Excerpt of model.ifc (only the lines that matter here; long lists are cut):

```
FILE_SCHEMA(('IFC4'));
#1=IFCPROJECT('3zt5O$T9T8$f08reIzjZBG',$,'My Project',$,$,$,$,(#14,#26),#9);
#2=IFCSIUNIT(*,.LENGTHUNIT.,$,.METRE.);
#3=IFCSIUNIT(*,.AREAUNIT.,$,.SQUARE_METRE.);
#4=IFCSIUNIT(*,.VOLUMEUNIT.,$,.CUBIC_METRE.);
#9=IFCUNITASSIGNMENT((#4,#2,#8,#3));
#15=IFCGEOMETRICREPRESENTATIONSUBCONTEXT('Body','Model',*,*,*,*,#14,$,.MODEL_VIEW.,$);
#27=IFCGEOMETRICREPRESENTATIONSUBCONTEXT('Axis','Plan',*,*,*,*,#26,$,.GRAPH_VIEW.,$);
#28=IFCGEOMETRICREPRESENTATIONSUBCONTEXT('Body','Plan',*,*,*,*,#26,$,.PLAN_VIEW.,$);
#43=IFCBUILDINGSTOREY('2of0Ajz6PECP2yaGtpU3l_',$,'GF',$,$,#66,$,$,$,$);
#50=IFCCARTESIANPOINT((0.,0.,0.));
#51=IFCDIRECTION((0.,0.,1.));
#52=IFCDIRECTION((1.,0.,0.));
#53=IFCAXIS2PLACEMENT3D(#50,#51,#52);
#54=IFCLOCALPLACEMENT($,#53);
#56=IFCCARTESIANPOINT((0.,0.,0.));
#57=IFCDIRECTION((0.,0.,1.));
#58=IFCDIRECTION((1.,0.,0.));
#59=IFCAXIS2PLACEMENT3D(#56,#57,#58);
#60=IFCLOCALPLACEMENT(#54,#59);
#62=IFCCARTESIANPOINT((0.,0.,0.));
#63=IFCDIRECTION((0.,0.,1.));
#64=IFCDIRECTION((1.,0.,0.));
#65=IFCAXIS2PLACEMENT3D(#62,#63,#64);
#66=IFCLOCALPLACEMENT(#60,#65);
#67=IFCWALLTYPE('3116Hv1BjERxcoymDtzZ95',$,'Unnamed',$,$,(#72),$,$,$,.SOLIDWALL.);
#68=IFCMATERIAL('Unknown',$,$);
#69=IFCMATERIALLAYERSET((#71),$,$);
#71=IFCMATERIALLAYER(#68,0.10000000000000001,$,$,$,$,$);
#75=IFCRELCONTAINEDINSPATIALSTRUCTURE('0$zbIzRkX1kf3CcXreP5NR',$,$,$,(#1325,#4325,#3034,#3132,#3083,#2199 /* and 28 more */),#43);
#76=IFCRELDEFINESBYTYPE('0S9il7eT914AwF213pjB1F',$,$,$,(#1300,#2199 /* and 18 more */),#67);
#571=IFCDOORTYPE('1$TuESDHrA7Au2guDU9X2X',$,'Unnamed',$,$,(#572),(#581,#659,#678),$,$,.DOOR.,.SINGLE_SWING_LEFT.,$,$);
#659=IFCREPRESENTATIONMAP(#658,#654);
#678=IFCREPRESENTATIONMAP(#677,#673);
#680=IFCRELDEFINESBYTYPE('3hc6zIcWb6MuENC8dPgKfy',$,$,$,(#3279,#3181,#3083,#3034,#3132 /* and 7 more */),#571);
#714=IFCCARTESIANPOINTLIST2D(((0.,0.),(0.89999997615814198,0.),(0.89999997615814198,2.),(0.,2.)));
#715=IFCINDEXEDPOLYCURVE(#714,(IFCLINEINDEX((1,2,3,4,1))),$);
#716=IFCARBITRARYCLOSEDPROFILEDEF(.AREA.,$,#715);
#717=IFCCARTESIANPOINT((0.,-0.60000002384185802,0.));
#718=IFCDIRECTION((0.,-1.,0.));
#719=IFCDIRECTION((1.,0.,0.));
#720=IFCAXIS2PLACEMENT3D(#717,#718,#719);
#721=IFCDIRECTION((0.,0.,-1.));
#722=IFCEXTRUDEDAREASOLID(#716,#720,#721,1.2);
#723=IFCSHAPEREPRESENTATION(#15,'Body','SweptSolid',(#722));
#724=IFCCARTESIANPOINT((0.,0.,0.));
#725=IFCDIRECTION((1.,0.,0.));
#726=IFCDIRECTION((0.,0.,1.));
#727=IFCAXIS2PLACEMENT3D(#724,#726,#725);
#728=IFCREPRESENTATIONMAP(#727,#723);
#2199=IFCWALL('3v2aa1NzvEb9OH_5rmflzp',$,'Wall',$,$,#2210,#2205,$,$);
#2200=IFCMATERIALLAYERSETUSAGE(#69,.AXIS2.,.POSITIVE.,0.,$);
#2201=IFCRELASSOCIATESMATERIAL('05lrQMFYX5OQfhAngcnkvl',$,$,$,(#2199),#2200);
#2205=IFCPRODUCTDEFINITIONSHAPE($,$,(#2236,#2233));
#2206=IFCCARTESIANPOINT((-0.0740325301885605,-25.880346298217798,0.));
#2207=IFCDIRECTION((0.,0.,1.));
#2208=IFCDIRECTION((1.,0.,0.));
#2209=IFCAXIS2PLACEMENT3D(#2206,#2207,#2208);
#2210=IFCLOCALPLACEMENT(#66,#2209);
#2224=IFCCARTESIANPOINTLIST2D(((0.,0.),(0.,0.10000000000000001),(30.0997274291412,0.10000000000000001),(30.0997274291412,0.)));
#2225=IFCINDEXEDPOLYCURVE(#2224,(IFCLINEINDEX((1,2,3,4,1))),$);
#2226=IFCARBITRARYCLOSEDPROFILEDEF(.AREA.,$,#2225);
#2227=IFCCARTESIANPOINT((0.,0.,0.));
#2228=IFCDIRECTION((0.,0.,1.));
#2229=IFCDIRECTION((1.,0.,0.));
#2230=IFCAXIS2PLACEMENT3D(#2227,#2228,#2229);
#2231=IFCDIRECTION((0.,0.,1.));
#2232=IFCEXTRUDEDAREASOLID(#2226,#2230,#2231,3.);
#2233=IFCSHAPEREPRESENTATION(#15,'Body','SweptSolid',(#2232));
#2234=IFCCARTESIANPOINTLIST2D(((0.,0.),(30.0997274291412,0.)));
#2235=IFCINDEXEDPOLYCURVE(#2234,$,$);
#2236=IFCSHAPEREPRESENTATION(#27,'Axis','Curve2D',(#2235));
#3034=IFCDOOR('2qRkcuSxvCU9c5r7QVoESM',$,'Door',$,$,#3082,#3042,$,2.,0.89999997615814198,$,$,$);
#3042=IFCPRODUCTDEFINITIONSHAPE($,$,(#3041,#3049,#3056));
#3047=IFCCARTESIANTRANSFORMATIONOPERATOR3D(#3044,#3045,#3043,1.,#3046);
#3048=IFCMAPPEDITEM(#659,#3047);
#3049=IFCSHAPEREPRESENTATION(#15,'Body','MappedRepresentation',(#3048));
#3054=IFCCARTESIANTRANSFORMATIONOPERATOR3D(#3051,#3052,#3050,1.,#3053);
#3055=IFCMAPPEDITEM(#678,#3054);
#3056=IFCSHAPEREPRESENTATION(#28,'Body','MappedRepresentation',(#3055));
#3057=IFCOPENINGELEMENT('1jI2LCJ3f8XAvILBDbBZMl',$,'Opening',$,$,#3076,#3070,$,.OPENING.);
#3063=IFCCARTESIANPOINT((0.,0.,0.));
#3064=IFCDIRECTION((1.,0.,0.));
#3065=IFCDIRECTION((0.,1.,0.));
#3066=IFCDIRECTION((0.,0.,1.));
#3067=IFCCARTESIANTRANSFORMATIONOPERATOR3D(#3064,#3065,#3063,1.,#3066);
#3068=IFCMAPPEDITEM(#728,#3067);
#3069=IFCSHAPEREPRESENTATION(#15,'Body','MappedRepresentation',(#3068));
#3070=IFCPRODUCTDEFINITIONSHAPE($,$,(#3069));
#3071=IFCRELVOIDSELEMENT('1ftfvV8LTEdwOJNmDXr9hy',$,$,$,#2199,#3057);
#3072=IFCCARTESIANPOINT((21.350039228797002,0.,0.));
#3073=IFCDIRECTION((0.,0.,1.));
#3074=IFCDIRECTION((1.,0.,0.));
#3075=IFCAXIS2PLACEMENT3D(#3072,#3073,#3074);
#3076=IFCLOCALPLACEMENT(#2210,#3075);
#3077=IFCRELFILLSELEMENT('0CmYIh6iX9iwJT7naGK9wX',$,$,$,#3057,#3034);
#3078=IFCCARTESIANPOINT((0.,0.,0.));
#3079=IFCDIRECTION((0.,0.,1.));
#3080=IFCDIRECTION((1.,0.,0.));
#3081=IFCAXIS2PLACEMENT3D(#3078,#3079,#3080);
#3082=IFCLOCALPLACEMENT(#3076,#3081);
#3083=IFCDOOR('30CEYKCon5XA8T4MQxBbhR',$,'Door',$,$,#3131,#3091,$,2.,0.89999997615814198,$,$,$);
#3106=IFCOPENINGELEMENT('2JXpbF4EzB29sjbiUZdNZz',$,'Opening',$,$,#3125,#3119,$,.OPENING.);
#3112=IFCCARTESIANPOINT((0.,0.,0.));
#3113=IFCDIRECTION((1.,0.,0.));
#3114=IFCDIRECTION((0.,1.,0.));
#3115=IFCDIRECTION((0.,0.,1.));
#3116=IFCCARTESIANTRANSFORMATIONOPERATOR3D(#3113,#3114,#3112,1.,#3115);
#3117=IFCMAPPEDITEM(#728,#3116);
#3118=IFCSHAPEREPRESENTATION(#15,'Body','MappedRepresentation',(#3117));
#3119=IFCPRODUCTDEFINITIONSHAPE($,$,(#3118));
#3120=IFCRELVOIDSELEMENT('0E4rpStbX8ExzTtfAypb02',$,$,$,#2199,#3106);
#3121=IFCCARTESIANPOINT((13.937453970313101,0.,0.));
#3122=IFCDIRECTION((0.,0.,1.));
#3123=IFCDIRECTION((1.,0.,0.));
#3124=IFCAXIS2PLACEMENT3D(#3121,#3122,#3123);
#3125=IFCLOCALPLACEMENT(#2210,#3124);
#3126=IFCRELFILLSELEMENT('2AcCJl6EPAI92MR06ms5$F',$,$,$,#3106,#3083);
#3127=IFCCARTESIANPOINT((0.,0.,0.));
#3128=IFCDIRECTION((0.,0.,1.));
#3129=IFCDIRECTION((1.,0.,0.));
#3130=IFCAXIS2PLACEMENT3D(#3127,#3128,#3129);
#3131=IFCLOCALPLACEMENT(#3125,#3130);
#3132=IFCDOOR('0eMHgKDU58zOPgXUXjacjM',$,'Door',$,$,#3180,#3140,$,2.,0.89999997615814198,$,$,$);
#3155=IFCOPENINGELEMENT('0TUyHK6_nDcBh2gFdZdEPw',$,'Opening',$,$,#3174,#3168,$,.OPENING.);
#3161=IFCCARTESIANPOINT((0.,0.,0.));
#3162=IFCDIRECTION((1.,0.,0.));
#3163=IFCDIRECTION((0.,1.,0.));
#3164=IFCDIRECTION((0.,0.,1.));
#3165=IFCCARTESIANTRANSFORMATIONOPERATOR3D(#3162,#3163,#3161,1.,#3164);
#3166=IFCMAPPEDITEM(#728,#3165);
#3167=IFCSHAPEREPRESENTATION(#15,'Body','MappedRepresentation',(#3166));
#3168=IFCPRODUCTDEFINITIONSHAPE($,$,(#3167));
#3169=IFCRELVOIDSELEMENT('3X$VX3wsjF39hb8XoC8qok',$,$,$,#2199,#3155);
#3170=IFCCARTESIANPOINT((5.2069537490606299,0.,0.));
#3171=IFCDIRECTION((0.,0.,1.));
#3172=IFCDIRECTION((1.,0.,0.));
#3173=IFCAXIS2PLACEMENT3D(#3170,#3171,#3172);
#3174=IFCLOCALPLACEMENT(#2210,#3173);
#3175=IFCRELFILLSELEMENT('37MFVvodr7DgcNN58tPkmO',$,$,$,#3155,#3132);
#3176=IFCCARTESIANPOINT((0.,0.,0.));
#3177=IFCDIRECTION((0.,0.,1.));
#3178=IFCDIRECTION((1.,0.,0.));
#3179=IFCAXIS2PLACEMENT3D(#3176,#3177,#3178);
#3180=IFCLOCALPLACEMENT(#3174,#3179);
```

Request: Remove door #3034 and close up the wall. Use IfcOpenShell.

```python
import ifcopenshell
import ifcopenshell.api.feature
import ifcopenshell.api.root
import ifcopenshell.geom
import ifcopenshell.util.shape

model = ifcopenshell.open("model.ifc")
settings = ifcopenshell.geom.settings()


def volume(element):
    """Net volume in cubic metres, openings subtracted."""
    shape = ifcopenshell.geom.create_shape(settings, element)
    return ifcopenshell.util.shape.get_volume(shape.geometry)


door = model.by_guid("2qRkcuSxvCU9c5r7QVoESM")
opening = door.FillsVoids[0].RelatingOpeningElement
wall = opening.VoidsElements[0].RelatingBuildingElement
before = volume(wall)

ifcopenshell.api.root.remove_product(model, product=door)
ifcopenshell.api.feature.remove_feature(model, feature=opening)

after = volume(wall)

print(f"wall volume {before:.3f} -> {after:.3f} m3")

model.write("model-out.ifc")
```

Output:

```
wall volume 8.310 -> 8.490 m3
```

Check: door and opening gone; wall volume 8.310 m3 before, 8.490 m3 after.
